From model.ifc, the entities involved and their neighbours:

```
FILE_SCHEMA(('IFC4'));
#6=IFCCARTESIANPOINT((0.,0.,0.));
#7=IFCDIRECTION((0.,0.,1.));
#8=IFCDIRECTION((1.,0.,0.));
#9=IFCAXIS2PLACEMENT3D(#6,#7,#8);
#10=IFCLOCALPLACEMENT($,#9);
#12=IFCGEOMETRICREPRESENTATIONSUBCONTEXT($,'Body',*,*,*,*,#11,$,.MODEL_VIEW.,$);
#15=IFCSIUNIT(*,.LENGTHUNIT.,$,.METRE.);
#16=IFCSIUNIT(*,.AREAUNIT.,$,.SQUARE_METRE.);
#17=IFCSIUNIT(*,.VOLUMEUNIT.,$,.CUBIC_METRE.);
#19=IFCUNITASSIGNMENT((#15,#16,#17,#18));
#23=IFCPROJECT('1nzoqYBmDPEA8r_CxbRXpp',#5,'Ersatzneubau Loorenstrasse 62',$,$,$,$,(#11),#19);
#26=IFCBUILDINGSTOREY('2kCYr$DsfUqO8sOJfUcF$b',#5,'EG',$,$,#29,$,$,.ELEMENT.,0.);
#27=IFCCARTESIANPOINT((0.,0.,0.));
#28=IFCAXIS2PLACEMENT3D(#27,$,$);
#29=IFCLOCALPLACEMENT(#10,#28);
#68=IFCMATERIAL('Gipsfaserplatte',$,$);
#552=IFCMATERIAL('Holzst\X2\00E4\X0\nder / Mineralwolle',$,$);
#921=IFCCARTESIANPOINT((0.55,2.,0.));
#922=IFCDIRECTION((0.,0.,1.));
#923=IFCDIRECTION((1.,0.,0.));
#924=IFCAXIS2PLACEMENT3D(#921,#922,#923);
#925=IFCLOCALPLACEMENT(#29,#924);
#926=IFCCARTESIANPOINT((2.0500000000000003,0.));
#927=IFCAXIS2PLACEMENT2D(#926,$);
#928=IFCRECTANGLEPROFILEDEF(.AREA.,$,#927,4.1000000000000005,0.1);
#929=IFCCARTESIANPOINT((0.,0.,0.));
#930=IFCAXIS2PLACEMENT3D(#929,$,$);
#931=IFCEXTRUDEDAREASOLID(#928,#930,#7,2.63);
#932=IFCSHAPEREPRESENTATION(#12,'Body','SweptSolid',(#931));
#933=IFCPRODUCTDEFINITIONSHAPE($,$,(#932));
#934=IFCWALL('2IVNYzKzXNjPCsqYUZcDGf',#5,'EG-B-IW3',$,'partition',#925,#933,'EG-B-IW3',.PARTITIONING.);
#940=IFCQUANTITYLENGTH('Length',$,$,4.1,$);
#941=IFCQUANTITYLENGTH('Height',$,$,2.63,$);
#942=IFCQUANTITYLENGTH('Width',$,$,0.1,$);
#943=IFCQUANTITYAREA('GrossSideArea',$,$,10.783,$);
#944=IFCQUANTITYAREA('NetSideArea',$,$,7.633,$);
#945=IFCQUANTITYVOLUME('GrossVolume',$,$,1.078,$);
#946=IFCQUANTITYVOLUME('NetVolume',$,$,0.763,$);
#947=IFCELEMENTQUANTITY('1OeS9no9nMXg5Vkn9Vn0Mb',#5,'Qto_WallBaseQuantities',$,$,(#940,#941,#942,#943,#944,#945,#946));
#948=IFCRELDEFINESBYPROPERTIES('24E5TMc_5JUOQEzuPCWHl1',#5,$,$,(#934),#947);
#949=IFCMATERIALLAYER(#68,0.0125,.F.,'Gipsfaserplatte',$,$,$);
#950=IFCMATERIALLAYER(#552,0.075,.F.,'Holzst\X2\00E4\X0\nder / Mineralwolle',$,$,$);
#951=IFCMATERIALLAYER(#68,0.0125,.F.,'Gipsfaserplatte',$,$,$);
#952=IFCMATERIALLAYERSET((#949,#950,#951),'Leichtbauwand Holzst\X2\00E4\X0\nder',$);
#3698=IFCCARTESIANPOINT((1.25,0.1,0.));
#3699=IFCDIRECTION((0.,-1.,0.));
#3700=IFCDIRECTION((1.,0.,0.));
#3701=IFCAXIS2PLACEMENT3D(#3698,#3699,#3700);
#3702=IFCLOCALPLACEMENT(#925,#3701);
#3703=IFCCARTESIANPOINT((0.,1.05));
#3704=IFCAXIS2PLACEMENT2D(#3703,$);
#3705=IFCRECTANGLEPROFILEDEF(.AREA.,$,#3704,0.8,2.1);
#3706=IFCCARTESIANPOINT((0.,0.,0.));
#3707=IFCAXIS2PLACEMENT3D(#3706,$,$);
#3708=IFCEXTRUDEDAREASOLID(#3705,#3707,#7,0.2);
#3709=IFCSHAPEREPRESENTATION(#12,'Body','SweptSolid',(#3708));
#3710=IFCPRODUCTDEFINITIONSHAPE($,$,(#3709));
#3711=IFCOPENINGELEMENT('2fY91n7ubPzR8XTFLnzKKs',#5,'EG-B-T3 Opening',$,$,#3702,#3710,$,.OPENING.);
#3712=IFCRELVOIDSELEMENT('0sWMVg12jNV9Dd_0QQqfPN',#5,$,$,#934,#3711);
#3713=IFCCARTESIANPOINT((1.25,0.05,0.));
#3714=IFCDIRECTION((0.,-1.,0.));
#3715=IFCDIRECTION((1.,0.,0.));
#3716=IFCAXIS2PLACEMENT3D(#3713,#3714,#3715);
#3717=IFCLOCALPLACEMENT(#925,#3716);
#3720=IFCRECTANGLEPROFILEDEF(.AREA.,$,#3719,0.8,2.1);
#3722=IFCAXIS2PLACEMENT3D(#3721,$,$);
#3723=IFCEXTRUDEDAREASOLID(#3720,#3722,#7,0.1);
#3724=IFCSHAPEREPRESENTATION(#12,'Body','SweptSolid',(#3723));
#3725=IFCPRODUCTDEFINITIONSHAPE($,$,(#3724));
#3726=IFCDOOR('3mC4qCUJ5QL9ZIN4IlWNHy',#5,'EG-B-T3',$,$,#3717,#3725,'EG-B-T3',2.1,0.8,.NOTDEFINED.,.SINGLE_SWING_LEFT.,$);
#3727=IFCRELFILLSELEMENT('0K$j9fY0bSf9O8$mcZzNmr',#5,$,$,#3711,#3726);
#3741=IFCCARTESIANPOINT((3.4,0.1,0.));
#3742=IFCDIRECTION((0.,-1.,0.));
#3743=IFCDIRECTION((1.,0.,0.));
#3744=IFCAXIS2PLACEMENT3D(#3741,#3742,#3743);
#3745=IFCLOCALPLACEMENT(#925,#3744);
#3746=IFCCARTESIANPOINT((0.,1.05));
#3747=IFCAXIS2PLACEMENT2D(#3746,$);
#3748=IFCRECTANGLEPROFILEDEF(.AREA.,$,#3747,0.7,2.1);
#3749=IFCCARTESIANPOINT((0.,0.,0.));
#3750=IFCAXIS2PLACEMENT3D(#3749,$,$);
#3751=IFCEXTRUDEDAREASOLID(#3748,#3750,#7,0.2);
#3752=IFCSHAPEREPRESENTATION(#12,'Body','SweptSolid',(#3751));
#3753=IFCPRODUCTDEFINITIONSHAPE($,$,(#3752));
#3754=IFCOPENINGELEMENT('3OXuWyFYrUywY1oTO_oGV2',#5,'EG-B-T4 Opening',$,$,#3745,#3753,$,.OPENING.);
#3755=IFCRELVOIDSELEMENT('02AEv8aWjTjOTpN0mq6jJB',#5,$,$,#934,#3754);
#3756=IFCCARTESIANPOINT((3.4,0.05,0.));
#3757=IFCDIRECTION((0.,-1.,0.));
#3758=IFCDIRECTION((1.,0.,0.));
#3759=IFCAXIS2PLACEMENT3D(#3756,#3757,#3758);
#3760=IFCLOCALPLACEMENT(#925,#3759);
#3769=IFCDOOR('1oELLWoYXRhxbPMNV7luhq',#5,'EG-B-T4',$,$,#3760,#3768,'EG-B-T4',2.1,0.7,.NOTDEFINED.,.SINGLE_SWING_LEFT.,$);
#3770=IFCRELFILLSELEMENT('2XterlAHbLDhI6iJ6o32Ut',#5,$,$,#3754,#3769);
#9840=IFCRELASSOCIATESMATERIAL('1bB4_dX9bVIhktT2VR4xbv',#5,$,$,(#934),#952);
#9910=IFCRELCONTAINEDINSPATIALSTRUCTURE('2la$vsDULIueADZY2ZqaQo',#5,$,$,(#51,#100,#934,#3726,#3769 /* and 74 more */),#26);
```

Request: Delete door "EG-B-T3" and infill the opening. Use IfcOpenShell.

```python
import ifcopenshell
import ifcopenshell.api.feature
import ifcopenshell.api.pset
import ifcopenshell.api.root
import ifcopenshell.geom
import ifcopenshell.util.element
import ifcopenshell.util.shape
import ifcopenshell.util.unit

model = ifcopenshell.open("model.ifc")
area_scale = ifcopenshell.util.unit.calculate_unit_scale(model, "AREAUNIT")
volume_scale = ifcopenshell.util.unit.calculate_unit_scale(model, "VOLUMEUNIT")
settings = ifcopenshell.geom.settings()


def volume(element):
    """Net volume in cubic metres, openings subtracted."""
    shape = ifcopenshell.geom.create_shape(settings, element)
    return ifcopenshell.util.shape.get_volume(shape.geometry)


door = model.by_guid("3mC4qCUJ5QL9ZIN4IlWNHy")
opening = door.FillsVoids[0].RelatingOpeningElement
wall = opening.VoidsElements[0].RelatingBuildingElement
before = volume(wall)

ifcopenshell.api.root.remove_product(model, product=door)
ifcopenshell.api.feature.remove_feature(model, feature=opening)

after = volume(wall)
thickness = 0.1  # wall thickness in metres

# Update the wall's stored quantities.
qto = model.by_id(ifcopenshell.util.element.get_pset(wall, "Qto_WallBaseQuantities", should_inherit=False)["id"])
ifcopenshell.api.pset.edit_qto(model, qto=qto, properties={
    "NetSideArea": after / thickness / area_scale,
    "NetVolume": after / volume_scale,
})

print(f"wall volume {before:.3f} -> {after:.3f} m3")

model.write("model_updated.ifc")
```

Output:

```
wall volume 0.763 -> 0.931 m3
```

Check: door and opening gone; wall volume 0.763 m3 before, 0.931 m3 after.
